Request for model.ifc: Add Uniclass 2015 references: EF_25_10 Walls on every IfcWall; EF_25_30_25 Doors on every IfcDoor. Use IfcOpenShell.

First a look at what the model holds.

```python
import ifcopenshell

model = ifcopenshell.open("model.ifc")
print(model.schema)
print("classifications:", [c.Name for c in model.by_type("IfcClassification")])
for ifc_class in ("IfcDoor", "IfcRoof", "IfcStair", "IfcWall", "IfcWindow"):
    print(ifc_class, len(model.by_type(ifc_class)))
```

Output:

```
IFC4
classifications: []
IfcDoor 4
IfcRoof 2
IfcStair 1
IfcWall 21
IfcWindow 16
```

```python
import ifcopenshell
import ifcopenshell.api.classification

model = ifcopenshell.open("model.ifc")

system = ifcopenshell.api.classification.add_classification(model, classification="Uniclass 2015")

codes = {
    "IfcWall": ("EF_25_10", "Walls"),
    "IfcDoor": ("EF_25_30_25", "Doors"),
}
for ifc_class, (code, name) in codes.items():
    products = model.by_type(ifc_class)
    ifcopenshell.api.classification.add_reference(
        model, products=products, classification=system, identification=code, name=name
    )
    print(code, len(products))

model.write("model_v2.ifc")
```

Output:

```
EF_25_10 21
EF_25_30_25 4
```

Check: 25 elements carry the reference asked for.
